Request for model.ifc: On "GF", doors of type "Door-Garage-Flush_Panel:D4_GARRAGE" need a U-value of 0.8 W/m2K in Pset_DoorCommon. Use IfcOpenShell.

First a look at what the model holds.

```python
import ifcopenshell
import ifcopenshell.util.element

model = ifcopenshell.open("model.ifc")
print(model.schema)
storey = next(s for s in model.by_type("IfcBuildingStorey") if s.Name == "GF")
doors = [e for e in ifcopenshell.util.element.get_decomposition(storey) if e.is_a("IfcDoor")]
seen = {}
for e in doors:
    element_type = ifcopenshell.util.element.get_type(e)
    key = (element_type.Name if element_type != e and element_type else None, ifcopenshell.util.element.get_pset(e, "Pset_DoorCommon", "ThermalTransmittance"))
    seen[key] = seen.get(key, 0) + 1
for (name, value), count in sorted(seen.items(), key=str):
    print(count, "x", name, "|", value)
```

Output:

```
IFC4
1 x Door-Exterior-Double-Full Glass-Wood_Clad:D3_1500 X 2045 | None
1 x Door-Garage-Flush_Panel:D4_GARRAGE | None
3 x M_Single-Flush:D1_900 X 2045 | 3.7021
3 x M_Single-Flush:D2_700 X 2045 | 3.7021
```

```python
import ifcopenshell
import ifcopenshell.api.pset
import ifcopenshell.util.element

model = ifcopenshell.open("model.ifc")

storey = next(s for s in model.by_type("IfcBuildingStorey") if s.Name == "GF")
doors = [e for e in ifcopenshell.util.element.get_decomposition(storey) if e.is_a("IfcDoor")]

count = 0
for e in doors:
    element_type = ifcopenshell.util.element.get_type(e)
    if element_type in (None, e) or element_type.Name != "Door-Garage-Flush_Panel:D4_GARRAGE":
        continue
    # add_pset returns the element's existing set when there is one.
    pset = ifcopenshell.api.pset.add_pset(model, product=e, name="Pset_DoorCommon")
    ifcopenshell.api.pset.edit_pset(model, pset=pset, properties={"ThermalTransmittance": 0.8})
    count += 1

print(count, "doors updated")

model.write("model_v2.ifc")
```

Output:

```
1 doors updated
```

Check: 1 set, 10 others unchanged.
